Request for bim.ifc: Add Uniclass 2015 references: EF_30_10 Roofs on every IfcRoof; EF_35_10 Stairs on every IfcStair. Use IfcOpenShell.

First a look at what the model holds.

```python
import ifcopenshell

model = ifcopenshell.open("bim.ifc")
print(model.schema)
print("classifications:", [c.Name for c in model.by_type("IfcClassification")])
for ifc_class in ("IfcDoor", "IfcRoof", "IfcStair", "IfcWall", "IfcWindow"):
    print(ifc_class, len(model.by_type(ifc_class)))
```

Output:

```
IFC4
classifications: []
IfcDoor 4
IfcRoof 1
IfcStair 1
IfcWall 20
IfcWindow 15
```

```python
import ifcopenshell
import ifcopenshell.api.classification

model = ifcopenshell.open("bim.ifc")

system = ifcopenshell.api.classification.add_classification(model, classification="Uniclass 2015")

codes = {
    "IfcRoof": ("EF_30_10", "Roofs"),
    "IfcStair": ("EF_35_10", "Stairs"),
}
for ifc_class, (code, name) in codes.items():
    products = model.by_type(ifc_class)
    ifcopenshell.api.classification.add_reference(
        model, products=products, classification=system, identification=code, name=name
    )
    print(code, len(products))

model.write("bim_v2.ifc")
```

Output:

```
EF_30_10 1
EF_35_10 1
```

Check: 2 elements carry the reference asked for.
